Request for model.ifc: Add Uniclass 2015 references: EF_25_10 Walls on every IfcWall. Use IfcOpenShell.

First a look at what the model holds.

```python
import ifcopenshell

model = ifcopenshell.open("model.ifc")
print(model.schema)
print("classifications:", [c.Name for c in model.by_type("IfcClassification")])
for ifc_class in ("IfcDoor", "IfcRoof", "IfcStair", "IfcWall", "IfcWindow"):
    print(ifc_class, len(model.by_type(ifc_class)))
```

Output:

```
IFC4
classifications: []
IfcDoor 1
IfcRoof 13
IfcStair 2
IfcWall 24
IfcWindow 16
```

```python
import ifcopenshell
import ifcopenshell.api.classification

model = ifcopenshell.open("model.ifc")

system = ifcopenshell.api.classification.add_classification(model, classification="Uniclass 2015")

codes = {
    "IfcWall": ("EF_25_10", "Walls"),
}
for ifc_class, (code, name) in codes.items():
    products = model.by_type(ifc_class)
    ifcopenshell.api.classification.add_reference(
        model, products=products, classification=system, identification=code, name=name
    )
    print(code, len(products))

model.write("model_v2.ifc")
```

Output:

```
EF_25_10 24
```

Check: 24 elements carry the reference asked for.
